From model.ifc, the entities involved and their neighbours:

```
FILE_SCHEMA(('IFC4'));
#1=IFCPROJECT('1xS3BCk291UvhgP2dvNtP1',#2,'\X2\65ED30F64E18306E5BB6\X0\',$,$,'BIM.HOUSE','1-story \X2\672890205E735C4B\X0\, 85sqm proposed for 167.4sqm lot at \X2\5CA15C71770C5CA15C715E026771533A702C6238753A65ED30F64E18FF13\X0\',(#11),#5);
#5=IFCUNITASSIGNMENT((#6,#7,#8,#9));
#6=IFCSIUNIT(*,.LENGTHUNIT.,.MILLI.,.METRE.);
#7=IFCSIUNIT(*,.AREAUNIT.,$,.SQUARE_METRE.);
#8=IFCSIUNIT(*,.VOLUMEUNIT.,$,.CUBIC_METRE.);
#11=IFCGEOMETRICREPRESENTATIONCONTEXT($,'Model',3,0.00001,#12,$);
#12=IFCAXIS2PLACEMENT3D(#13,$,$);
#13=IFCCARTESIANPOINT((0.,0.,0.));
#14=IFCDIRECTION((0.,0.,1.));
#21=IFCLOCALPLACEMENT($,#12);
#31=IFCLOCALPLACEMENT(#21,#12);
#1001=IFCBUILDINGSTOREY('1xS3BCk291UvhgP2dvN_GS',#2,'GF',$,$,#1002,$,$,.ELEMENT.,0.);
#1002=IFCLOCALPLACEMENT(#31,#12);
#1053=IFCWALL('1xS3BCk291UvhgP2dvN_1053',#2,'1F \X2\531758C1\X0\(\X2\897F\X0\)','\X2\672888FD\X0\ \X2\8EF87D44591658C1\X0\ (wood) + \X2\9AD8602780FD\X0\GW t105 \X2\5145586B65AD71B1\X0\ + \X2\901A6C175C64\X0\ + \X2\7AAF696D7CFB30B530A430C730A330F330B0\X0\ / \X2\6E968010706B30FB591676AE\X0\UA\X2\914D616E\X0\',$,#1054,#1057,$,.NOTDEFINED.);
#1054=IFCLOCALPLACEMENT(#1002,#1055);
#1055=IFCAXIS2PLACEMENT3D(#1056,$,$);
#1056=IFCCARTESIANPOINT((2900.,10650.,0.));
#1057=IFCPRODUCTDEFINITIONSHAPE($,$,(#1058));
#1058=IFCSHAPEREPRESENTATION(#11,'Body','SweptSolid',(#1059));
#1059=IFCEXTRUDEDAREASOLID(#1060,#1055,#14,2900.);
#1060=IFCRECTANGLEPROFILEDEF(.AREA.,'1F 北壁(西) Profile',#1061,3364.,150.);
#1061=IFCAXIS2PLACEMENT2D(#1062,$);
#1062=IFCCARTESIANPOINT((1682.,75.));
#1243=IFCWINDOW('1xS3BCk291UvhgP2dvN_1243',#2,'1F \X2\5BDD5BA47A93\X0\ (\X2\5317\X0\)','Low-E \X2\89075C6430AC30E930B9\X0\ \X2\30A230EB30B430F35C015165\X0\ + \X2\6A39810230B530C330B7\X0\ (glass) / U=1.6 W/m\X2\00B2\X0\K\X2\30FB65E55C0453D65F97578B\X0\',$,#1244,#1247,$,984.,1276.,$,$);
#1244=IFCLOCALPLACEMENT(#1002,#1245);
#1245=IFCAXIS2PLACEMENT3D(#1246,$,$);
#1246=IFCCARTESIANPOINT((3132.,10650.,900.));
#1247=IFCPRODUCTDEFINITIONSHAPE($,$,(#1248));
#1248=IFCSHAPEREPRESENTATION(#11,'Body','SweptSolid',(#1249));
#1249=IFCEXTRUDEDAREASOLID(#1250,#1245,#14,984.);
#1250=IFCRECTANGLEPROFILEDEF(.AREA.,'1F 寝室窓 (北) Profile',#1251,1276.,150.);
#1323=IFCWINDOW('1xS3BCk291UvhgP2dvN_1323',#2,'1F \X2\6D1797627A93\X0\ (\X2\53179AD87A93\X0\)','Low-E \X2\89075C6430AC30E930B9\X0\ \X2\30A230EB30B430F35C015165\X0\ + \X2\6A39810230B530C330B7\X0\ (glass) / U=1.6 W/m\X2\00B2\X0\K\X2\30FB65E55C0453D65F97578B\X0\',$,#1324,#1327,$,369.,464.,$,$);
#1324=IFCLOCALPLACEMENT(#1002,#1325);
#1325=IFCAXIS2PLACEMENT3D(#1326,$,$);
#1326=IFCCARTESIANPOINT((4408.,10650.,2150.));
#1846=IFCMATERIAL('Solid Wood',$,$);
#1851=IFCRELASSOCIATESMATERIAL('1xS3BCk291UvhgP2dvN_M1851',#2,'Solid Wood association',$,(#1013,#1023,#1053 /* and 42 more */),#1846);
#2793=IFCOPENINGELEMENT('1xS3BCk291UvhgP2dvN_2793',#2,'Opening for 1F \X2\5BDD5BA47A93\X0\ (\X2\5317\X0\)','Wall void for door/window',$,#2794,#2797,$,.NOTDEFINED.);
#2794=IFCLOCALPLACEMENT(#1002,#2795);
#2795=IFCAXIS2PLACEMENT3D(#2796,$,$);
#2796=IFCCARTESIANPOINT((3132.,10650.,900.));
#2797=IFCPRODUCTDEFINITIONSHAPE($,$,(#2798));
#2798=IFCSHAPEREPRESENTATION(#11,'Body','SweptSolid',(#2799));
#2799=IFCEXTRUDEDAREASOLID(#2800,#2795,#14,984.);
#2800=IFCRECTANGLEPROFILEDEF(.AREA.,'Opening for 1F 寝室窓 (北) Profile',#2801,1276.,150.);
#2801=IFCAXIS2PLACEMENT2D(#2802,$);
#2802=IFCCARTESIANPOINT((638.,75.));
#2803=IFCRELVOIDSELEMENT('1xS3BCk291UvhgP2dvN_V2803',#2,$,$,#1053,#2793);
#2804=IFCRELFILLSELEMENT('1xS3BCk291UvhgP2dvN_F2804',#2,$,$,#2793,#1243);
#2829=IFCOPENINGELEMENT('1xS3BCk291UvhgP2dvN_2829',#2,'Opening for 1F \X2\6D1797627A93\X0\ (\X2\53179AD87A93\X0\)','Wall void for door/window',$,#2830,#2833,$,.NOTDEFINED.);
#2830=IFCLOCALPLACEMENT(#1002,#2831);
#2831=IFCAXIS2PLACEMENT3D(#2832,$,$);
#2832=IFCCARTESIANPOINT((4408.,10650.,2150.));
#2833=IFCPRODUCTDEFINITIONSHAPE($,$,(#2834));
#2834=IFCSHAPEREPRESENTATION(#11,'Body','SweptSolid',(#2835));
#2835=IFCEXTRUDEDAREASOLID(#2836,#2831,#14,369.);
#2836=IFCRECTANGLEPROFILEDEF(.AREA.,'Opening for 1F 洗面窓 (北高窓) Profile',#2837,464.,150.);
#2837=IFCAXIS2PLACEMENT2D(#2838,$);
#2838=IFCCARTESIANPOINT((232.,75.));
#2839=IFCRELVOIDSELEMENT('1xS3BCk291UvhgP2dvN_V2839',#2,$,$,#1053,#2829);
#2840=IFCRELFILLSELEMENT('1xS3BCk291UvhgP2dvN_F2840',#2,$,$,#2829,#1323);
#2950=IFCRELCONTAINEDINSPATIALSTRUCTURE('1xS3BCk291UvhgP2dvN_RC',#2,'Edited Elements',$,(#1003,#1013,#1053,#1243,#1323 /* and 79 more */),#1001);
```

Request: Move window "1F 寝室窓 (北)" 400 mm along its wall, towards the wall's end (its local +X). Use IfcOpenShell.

```python
import ifcopenshell
import ifcopenshell.api.geometry
import ifcopenshell.util.placement
import ifcopenshell.util.unit

model = ifcopenshell.open("model.ifc")
unit_scale = ifcopenshell.util.unit.calculate_unit_scale(model)

window = model.by_id(1243)
opening = window.FillsVoids[0].RelatingOpeningElement
wall = opening.VoidsElements[0].RelatingBuildingElement

wall_matrix = ifcopenshell.util.placement.get_local_placement(wall.ObjectPlacement)
shift = wall_matrix[:3, 0] * 0.4 / unit_scale
before = ifcopenshell.util.placement.get_local_placement(window.ObjectPlacement)[:3, 3].copy()

# The window is not placed relative to its opening, so move both.
for product in (opening, window):
    matrix = ifcopenshell.util.placement.get_local_placement(product.ObjectPlacement)
    matrix[:3, 3] += shift
    ifcopenshell.api.geometry.edit_object_placement(model, product=product, matrix=matrix, is_si=False)

after = ifcopenshell.util.placement.get_local_placement(window.ObjectPlacement)[:3, 3]
print("window moved by", (after - before).round(3) + 0.0)

model.write("model-out.ifc")
```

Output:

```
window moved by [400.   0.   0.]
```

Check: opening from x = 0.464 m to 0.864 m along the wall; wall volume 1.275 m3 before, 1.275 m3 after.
